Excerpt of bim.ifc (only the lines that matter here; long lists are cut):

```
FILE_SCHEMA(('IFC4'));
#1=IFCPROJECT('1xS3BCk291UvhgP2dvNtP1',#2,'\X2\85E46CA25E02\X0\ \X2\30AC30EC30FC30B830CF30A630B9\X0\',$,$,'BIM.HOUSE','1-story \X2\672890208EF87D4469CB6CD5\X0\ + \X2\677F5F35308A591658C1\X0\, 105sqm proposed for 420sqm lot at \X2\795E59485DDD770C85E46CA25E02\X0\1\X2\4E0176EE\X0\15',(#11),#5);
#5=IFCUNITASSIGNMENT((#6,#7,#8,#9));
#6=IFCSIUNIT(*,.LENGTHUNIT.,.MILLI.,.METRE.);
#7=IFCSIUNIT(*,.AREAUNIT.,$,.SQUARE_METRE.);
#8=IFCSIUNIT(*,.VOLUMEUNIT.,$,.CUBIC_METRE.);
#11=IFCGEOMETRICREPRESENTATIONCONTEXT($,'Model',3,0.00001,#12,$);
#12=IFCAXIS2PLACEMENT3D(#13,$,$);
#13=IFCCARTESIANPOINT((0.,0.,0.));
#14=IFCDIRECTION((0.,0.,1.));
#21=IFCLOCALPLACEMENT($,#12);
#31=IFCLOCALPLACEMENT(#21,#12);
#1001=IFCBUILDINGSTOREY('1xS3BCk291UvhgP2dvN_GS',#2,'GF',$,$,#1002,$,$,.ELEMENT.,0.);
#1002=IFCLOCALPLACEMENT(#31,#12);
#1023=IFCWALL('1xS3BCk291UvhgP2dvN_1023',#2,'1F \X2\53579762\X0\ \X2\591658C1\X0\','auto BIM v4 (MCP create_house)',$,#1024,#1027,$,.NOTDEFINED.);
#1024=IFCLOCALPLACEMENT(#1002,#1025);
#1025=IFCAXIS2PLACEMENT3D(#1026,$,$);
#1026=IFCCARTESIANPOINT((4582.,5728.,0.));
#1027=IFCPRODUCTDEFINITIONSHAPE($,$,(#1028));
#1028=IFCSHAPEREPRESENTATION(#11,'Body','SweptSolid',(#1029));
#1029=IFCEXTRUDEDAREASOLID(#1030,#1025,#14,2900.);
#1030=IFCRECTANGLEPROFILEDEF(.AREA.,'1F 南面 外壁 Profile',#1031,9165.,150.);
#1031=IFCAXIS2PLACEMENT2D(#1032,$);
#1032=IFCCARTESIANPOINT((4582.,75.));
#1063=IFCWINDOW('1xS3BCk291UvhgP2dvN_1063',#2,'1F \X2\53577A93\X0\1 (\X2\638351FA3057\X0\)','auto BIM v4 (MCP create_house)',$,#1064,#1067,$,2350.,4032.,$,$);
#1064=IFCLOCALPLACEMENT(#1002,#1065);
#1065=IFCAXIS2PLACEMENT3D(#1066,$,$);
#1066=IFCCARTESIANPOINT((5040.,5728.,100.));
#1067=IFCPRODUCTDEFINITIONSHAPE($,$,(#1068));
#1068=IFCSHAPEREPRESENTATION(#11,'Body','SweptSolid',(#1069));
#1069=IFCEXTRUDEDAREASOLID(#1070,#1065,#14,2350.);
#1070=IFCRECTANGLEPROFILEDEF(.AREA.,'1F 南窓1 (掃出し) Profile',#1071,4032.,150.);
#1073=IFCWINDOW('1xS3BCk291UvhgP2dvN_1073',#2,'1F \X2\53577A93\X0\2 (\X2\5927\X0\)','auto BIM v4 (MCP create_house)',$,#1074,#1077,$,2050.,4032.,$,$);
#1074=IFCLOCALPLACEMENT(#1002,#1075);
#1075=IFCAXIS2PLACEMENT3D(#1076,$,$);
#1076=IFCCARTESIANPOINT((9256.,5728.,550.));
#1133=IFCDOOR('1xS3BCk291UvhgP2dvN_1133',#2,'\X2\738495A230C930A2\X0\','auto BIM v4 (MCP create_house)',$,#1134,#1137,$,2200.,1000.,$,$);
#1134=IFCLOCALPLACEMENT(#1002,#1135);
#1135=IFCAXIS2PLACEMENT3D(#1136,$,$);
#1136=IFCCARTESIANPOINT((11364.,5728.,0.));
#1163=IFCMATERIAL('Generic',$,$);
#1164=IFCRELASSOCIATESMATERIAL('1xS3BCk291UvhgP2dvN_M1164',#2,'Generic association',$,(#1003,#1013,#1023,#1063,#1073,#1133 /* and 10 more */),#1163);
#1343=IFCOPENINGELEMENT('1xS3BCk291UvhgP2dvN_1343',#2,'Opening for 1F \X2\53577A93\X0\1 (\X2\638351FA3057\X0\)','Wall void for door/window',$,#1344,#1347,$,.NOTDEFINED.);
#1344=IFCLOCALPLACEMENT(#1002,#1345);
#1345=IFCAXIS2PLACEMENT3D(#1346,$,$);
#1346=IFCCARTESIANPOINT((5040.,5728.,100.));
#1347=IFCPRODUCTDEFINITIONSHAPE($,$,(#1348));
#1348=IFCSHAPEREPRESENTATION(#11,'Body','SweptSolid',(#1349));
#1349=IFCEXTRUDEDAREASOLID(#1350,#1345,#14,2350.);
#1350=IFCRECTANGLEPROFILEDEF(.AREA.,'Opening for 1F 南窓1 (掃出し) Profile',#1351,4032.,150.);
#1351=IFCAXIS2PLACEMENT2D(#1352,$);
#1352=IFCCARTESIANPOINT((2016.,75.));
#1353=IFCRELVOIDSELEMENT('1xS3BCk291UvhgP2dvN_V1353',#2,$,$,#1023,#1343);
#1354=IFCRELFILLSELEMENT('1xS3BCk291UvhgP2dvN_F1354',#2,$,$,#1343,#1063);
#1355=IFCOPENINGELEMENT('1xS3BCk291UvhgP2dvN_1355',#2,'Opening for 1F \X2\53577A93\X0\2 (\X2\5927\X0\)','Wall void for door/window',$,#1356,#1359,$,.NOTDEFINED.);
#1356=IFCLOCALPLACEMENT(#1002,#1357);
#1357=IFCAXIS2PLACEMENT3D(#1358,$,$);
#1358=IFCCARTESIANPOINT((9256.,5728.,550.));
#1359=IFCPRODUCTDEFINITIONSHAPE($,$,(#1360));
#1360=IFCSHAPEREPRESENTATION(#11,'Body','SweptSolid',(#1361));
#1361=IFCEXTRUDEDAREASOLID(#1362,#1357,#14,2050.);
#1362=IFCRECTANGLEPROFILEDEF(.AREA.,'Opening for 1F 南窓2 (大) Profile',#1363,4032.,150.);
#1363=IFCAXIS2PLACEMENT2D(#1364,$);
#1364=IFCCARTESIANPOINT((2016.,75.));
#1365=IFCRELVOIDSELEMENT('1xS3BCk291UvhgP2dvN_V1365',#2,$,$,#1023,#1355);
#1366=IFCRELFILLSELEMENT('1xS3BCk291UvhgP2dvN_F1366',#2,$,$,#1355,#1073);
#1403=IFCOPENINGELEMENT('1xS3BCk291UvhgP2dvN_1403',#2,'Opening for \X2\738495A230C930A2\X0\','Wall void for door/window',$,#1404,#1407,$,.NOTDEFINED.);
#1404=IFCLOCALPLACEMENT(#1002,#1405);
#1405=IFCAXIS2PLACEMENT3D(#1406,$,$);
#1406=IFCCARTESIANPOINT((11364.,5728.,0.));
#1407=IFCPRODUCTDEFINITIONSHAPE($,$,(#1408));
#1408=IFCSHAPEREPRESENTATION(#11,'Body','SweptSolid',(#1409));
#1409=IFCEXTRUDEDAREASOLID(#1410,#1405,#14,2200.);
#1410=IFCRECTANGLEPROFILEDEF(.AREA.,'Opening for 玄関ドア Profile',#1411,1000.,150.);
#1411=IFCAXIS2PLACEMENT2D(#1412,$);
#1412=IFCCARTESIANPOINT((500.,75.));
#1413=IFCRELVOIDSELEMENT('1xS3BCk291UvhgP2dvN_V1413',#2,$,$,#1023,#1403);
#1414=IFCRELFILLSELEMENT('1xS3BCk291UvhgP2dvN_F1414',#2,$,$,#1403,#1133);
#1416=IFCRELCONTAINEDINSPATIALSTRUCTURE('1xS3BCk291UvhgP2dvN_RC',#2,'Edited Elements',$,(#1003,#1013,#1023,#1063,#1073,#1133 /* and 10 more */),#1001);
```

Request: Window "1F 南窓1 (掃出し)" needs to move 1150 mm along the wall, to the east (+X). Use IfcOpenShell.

```python
import ifcopenshell
import ifcopenshell.api.geometry
import ifcopenshell.util.placement

model = ifcopenshell.open("bim.ifc")

window = model.by_id(1063)
opening = window.FillsVoids[0].RelatingOpeningElement
wall = opening.VoidsElements[0].RelatingBuildingElement

wall_matrix = ifcopenshell.util.placement.get_local_placement(wall.ObjectPlacement)
shift = wall_matrix[:3, 0] * 1150.0
before = ifcopenshell.util.placement.get_local_placement(window.ObjectPlacement)[:3, 3].copy()

# The window is not placed relative to its opening, so move both.
for product in (opening, window):
    matrix = ifcopenshell.util.placement.get_local_placement(product.ObjectPlacement)
    matrix[:3, 3] += shift
    ifcopenshell.api.geometry.edit_object_placement(model, product=product, matrix=matrix, is_si=False)

after = ifcopenshell.util.placement.get_local_placement(window.ObjectPlacement)[:3, 3]
print("window moved by", (after - before).round(3) + 0.0)

model.write("bim_rev.ifc")
```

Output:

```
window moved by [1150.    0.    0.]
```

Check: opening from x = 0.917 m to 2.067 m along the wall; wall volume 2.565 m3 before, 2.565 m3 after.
